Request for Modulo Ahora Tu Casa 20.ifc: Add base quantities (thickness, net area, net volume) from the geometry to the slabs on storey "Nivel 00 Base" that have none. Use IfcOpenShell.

First a look at what the model holds.

```python
import ifcopenshell
import ifcopenshell.util.element
import ifcopenshell.util.unit

model = ifcopenshell.open("Modulo Ahora Tu Casa 20.ifc")
print(model.schema)
for unit_type in ("LENGTHUNIT", "AREAUNIT", "VOLUMEUNIT"):
    print(unit_type, ifcopenshell.util.unit.calculate_unit_scale(model, unit_type))
storey = next(s for s in model.by_type("IfcBuildingStorey") if s.Name == "Nivel 00 Base")
slabs = [e for e in ifcopenshell.util.element.get_decomposition(storey) if e.is_a("IfcSlab")]
for e in sorted(slabs, key=lambda e: e.id()):
    print(e.id(), e.is_a(), e.Name, list(ifcopenshell.util.element.get_psets(e, qtos_only=True)), sep=" | ")
```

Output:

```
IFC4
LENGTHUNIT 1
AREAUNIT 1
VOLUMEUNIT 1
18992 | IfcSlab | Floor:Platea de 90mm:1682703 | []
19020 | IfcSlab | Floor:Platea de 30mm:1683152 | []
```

```python
import ifcopenshell
import ifcopenshell.api.pset
import ifcopenshell.geom
import ifcopenshell.util.element
import ifcopenshell.util.shape
import ifcopenshell.util.unit

model = ifcopenshell.open("Modulo Ahora Tu Casa 20.ifc")
unit_scale = ifcopenshell.util.unit.calculate_unit_scale(model)
area_scale = ifcopenshell.util.unit.calculate_unit_scale(model, "AREAUNIT")
volume_scale = ifcopenshell.util.unit.calculate_unit_scale(model, "VOLUMEUNIT")
settings = ifcopenshell.geom.settings()

storey = next(s for s in model.by_type("IfcBuildingStorey") if s.Name == "Nivel 00 Base")
slabs = [e for e in ifcopenshell.util.element.get_decomposition(storey) if e.is_a("IfcSlab")]

for e in sorted(slabs, key=lambda e: e.id()):
    if ifcopenshell.util.element.get_psets(e, qtos_only=True, should_inherit=False):
        continue
    # Geometry comes back in metres, in the element's own axes.
    shape = ifcopenshell.geom.create_shape(settings, e)
    values = {
        "Width": ifcopenshell.util.shape.get_z(shape.geometry) / unit_scale,
        "NetArea": ifcopenshell.util.shape.get_footprint_area(shape.geometry) / area_scale,
        "NetVolume": ifcopenshell.util.shape.get_volume(shape.geometry) / volume_scale,
    }
    qto = ifcopenshell.api.pset.add_qto(model, product=e, name="Qto_SlabBaseQuantities")
    ifcopenshell.api.pset.edit_qto(model, qto=qto, properties=values)
    print(e.id(), {k: round(v, 3) for k, v in values.items()})

model.write("Modulo Ahora Tu Casa 20_edited.ifc")
```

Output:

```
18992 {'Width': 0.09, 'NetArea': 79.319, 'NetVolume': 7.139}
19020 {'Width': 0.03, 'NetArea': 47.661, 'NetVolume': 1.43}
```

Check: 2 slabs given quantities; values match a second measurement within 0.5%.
